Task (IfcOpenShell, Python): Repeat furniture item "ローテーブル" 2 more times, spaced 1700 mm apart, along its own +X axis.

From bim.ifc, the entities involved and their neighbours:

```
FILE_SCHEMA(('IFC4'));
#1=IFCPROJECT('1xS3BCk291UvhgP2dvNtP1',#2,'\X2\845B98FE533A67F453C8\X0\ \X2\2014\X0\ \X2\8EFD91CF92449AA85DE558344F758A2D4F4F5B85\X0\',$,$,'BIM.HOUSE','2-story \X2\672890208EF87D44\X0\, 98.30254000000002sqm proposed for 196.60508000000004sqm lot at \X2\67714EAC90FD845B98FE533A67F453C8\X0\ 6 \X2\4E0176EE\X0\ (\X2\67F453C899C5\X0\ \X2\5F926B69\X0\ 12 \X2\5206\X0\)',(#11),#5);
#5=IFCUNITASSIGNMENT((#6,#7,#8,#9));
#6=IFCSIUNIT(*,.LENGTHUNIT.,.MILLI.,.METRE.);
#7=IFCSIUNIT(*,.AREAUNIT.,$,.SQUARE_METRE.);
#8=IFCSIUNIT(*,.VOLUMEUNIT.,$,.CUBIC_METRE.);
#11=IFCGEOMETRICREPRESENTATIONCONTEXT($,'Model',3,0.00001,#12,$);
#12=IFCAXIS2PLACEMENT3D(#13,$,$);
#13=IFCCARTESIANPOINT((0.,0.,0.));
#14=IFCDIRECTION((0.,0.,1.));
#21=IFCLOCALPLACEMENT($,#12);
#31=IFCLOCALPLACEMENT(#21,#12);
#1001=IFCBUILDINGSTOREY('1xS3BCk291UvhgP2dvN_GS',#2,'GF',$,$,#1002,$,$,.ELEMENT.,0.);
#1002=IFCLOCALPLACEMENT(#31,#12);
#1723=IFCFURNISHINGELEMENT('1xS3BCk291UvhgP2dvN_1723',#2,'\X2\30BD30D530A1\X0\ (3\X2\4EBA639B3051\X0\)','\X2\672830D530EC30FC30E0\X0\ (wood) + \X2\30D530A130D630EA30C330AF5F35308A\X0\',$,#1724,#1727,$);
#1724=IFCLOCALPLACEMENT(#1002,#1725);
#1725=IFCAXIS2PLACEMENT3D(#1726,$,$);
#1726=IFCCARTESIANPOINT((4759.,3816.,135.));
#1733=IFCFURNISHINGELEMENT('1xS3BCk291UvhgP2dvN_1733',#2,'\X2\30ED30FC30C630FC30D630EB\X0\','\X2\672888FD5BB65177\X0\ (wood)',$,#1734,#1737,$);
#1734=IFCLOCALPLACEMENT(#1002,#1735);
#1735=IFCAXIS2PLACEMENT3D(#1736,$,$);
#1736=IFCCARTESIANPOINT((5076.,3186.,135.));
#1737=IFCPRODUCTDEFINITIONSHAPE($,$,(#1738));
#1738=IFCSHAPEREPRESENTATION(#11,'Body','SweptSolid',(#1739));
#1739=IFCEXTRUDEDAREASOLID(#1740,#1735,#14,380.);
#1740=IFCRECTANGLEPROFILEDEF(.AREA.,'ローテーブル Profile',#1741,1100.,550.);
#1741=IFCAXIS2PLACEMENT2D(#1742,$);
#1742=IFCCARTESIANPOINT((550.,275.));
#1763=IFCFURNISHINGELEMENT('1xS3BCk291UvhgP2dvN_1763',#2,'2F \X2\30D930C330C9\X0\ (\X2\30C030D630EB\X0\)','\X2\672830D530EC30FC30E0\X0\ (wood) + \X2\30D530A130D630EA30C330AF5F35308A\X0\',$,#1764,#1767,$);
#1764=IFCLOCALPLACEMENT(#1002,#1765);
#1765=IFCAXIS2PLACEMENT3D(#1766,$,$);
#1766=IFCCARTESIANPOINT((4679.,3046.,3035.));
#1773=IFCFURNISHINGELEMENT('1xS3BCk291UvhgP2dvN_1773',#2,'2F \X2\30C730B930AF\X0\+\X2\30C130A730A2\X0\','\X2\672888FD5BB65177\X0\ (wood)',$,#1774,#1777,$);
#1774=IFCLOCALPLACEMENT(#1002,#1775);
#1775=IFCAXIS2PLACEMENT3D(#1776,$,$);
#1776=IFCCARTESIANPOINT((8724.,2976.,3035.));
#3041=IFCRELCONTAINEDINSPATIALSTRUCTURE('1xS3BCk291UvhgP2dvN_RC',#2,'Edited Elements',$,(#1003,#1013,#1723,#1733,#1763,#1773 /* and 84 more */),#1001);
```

```python
import ifcopenshell
import ifcopenshell.api.geometry
import ifcopenshell.api.root
import ifcopenshell.util.element
import ifcopenshell.util.placement

model = ifcopenshell.open("bim.ifc")


def reuse_history(source, copy):
    """copy_class also copies each property set's owner history, people and application; keep the originals."""
    for rel in copy.IsDefinedBy:
        if rel.is_a("IfcRelDefinesByProperties") and (history := rel.RelatingPropertyDefinition.OwnerHistory):
            rel.RelatingPropertyDefinition.OwnerHistory = source.OwnerHistory
            ifcopenshell.util.element.remove_deep2(model, history)


source = model.by_guid("1xS3BCk291UvhgP2dvN_1733")
base = ifcopenshell.util.placement.get_local_placement(source.ObjectPlacement)
step = base[:3, 0] * 1700.0

for i in range(1, 3):
    copy = ifcopenshell.api.root.copy_class(model, product=source)
    copy.Representation = ifcopenshell.util.element.copy_deep(
        model, source.Representation, exclude=["IfcGeometricRepresentationContext", "IfcRepresentationMap"]
    )
    reuse_history(source, copy)
    matrix = base.copy()
    matrix[:3, 3] += i * step
    print("added at", matrix[:3, 3].round(3) + 0.0)
    ifcopenshell.api.geometry.edit_object_placement(model, product=copy, matrix=matrix, is_si=False)

model.write("bim_edited.ifc")
```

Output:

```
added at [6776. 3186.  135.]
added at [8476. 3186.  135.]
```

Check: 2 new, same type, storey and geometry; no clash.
